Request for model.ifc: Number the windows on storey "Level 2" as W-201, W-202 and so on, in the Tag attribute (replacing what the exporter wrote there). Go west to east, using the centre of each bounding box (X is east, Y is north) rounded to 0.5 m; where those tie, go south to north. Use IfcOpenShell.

First a look at what the model holds.

```python
import ifcopenshell
import ifcopenshell.util.element
import ifcopenshell.util.placement

model = ifcopenshell.open("model.ifc")
print(model.schema)
storey = next(s for s in model.by_type("IfcBuildingStorey") if s.Name == "Level 2")
windows = [e for e in ifcopenshell.util.element.get_decomposition(storey) if e.is_a("IfcWindow")]
for e in sorted(windows, key=lambda e: e.id()):
    origin = ifcopenshell.util.placement.get_local_placement(e.ObjectPlacement)[:3, 3]
    print(e.id(), e.Tag, e.Name, origin.round(2) + 0.0, sep=" | ")
```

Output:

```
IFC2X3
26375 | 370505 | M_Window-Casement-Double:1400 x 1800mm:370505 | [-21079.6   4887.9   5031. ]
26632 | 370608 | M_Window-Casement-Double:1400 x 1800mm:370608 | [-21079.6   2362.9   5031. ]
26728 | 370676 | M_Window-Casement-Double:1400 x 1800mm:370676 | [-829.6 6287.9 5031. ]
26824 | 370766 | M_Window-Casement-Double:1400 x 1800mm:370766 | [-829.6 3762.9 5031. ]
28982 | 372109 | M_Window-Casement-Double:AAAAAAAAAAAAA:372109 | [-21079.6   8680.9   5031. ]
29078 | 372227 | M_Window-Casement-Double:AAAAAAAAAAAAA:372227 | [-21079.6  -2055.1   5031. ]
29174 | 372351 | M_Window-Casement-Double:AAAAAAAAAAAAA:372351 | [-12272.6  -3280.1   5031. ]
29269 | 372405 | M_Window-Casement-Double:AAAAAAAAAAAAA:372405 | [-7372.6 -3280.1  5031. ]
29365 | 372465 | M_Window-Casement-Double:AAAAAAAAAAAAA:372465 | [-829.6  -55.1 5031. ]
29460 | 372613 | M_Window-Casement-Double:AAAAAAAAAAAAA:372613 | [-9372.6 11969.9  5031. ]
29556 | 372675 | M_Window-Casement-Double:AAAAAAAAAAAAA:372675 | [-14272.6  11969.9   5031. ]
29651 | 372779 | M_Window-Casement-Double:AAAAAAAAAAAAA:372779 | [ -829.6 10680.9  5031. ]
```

```python
import ifcopenshell
import ifcopenshell.geom
import ifcopenshell.util.element
import ifcopenshell.util.shape

model = ifcopenshell.open("model.ifc")
settings = ifcopenshell.geom.settings()
settings.set("use-world-coords", True)


def centre(element):
    shape = ifcopenshell.geom.create_shape(settings, element)
    return ifcopenshell.util.shape.get_bbox_centroid(shape.geometry)


storey = next(s for s in model.by_type("IfcBuildingStorey") if s.Name == "Level 2")
windows = [e for e in ifcopenshell.util.element.get_decomposition(storey) if e.is_a("IfcWindow")]

# Insertion points can sit at a corner or the storey origin, so sort by the geometry (in metres).
centres = {e: centre(e) for e in windows}
windows.sort(key=lambda e: (round(centres[e][0] / 0.5), centres[e][1]))

for i, e in enumerate(windows, start=1):
    number = f"W-2{i:02d}"
    e.Tag = number
    print(e.id(), number)

model.write("model_rev.ifc")
```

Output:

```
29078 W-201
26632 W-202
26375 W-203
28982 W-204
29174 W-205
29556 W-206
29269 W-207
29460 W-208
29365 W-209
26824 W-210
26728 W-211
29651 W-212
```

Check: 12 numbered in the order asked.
